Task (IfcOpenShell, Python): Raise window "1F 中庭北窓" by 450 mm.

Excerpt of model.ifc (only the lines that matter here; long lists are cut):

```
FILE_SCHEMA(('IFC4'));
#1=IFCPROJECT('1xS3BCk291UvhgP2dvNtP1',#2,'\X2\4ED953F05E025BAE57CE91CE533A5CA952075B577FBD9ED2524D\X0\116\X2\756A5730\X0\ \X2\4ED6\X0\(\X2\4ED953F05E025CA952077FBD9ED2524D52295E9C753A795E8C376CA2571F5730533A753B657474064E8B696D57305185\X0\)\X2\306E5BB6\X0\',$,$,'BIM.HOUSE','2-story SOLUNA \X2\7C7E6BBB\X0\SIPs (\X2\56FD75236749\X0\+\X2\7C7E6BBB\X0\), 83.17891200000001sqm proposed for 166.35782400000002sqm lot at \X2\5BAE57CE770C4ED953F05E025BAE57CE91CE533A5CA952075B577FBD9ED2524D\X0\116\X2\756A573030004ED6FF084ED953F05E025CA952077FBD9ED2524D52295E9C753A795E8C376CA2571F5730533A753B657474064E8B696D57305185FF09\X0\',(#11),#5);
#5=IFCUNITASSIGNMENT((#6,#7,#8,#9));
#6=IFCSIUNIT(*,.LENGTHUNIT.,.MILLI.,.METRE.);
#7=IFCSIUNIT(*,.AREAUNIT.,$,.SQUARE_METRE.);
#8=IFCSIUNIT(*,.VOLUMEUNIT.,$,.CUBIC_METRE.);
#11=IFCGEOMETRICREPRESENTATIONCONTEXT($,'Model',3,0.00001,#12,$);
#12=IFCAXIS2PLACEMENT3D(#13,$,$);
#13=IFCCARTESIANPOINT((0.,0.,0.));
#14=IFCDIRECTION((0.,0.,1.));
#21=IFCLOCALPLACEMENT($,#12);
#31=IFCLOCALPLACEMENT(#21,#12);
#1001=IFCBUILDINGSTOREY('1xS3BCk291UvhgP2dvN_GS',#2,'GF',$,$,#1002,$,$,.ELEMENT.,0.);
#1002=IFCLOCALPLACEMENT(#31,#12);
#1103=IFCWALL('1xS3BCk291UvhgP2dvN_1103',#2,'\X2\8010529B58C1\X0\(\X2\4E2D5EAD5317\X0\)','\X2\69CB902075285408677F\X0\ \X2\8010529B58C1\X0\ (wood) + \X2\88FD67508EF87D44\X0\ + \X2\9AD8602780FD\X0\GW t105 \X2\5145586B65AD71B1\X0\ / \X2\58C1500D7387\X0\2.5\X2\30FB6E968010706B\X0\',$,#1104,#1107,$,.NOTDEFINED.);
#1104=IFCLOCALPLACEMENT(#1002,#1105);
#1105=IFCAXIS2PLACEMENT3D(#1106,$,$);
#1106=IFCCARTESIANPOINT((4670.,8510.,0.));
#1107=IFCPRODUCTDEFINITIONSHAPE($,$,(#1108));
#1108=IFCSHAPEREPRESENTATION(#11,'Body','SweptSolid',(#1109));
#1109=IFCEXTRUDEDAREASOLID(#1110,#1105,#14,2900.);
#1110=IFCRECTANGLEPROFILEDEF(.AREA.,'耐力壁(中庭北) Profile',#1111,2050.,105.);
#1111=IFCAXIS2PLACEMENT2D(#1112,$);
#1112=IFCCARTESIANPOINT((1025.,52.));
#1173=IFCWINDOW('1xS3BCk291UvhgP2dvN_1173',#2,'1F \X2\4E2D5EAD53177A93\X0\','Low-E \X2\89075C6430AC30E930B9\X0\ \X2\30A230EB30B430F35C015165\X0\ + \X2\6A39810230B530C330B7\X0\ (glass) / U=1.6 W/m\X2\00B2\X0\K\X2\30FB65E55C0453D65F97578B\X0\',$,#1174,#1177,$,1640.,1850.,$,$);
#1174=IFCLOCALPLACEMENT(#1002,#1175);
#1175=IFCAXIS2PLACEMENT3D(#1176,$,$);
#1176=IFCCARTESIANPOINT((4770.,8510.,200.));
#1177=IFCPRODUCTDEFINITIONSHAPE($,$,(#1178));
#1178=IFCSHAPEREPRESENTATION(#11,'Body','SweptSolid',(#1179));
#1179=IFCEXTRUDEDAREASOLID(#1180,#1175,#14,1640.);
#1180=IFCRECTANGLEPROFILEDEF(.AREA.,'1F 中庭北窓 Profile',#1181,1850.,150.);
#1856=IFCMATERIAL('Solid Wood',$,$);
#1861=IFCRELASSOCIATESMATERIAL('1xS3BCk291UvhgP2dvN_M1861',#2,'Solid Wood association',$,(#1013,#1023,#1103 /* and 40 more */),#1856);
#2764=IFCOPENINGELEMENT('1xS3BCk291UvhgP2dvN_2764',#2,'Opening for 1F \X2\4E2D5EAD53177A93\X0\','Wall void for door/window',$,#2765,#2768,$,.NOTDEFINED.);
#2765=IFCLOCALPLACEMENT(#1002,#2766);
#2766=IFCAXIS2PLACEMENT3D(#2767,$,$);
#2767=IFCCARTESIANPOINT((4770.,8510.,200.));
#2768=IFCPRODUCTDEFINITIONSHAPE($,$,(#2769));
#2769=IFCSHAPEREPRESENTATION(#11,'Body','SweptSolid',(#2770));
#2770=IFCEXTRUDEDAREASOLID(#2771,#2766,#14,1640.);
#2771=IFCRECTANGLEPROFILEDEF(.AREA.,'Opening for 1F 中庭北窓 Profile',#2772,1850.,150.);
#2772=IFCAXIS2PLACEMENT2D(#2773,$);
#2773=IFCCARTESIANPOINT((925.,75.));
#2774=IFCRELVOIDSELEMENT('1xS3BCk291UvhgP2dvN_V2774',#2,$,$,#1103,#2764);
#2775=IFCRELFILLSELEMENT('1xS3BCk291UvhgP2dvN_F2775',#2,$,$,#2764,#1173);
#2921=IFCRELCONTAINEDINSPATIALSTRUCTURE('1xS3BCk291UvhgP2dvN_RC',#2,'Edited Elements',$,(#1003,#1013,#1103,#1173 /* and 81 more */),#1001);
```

```python
import numpy as np
import ifcopenshell
import ifcopenshell.api.geometry
import ifcopenshell.util.placement
import ifcopenshell.util.unit

model = ifcopenshell.open("model.ifc")
unit_scale = ifcopenshell.util.unit.calculate_unit_scale(model)

window = model.by_guid("1xS3BCk291UvhgP2dvN_1173")
opening = window.FillsVoids[0].RelatingOpeningElement
dz = 0.45 / unit_scale

shift = np.array([0.0, 0.0, dz])
# The window is not placed relative to its opening, so move both.
for product in (opening, window):
    matrix = ifcopenshell.util.placement.get_local_placement(product.ObjectPlacement)
    matrix[:3, 3] += shift
    ifcopenshell.api.geometry.edit_object_placement(model, product=product, matrix=matrix, is_si=False)

print(f"moved by {dz * unit_scale:+.3f} m")

model.write("model_rev.ifc")
```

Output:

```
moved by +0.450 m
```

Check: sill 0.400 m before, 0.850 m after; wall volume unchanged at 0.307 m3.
